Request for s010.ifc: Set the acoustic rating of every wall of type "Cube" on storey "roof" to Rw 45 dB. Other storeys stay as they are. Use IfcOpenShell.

First a look at what the model holds.

```python
import ifcopenshell
import ifcopenshell.util.element

model = ifcopenshell.open("s010.ifc")
print(model.schema)
storey = next(s for s in model.by_type("IfcBuildingStorey") if s.Name == "roof")
walls = [e for e in ifcopenshell.util.element.get_decomposition(storey) if e.is_a("IfcWall")]
seen = {}
for e in walls:
    element_type = ifcopenshell.util.element.get_type(e)
    key = (element_type.Name if element_type != e and element_type else None, ifcopenshell.util.element.get_pset(e, "Pset_WallCommon", "AcousticRating"))
    seen[key] = seen.get(key, 0) + 1
for (name, value), count in sorted(seen.items(), key=str):
    print(count, "x", name, "|", value)
```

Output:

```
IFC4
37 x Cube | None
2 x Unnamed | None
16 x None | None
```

```python
import ifcopenshell
import ifcopenshell.api.pset
import ifcopenshell.util.element

model = ifcopenshell.open("s010.ifc")

storey = next(s for s in model.by_type("IfcBuildingStorey") if s.Name == "roof")
walls = [e for e in ifcopenshell.util.element.get_decomposition(storey) if e.is_a("IfcWall")]

count = 0
for e in walls:
    element_type = ifcopenshell.util.element.get_type(e)
    if element_type in (None, e) or element_type.Name != "Cube":
        continue
    # add_pset returns the element's existing set when there is one.
    pset = ifcopenshell.api.pset.add_pset(model, product=e, name="Pset_WallCommon")
    ifcopenshell.api.pset.edit_pset(model, pset=pset, properties={"AcousticRating": "Rw 45 dB"})
    count += 1

print(count, "walls updated")

model.write("s010_rev.ifc")
```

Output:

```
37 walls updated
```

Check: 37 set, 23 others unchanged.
